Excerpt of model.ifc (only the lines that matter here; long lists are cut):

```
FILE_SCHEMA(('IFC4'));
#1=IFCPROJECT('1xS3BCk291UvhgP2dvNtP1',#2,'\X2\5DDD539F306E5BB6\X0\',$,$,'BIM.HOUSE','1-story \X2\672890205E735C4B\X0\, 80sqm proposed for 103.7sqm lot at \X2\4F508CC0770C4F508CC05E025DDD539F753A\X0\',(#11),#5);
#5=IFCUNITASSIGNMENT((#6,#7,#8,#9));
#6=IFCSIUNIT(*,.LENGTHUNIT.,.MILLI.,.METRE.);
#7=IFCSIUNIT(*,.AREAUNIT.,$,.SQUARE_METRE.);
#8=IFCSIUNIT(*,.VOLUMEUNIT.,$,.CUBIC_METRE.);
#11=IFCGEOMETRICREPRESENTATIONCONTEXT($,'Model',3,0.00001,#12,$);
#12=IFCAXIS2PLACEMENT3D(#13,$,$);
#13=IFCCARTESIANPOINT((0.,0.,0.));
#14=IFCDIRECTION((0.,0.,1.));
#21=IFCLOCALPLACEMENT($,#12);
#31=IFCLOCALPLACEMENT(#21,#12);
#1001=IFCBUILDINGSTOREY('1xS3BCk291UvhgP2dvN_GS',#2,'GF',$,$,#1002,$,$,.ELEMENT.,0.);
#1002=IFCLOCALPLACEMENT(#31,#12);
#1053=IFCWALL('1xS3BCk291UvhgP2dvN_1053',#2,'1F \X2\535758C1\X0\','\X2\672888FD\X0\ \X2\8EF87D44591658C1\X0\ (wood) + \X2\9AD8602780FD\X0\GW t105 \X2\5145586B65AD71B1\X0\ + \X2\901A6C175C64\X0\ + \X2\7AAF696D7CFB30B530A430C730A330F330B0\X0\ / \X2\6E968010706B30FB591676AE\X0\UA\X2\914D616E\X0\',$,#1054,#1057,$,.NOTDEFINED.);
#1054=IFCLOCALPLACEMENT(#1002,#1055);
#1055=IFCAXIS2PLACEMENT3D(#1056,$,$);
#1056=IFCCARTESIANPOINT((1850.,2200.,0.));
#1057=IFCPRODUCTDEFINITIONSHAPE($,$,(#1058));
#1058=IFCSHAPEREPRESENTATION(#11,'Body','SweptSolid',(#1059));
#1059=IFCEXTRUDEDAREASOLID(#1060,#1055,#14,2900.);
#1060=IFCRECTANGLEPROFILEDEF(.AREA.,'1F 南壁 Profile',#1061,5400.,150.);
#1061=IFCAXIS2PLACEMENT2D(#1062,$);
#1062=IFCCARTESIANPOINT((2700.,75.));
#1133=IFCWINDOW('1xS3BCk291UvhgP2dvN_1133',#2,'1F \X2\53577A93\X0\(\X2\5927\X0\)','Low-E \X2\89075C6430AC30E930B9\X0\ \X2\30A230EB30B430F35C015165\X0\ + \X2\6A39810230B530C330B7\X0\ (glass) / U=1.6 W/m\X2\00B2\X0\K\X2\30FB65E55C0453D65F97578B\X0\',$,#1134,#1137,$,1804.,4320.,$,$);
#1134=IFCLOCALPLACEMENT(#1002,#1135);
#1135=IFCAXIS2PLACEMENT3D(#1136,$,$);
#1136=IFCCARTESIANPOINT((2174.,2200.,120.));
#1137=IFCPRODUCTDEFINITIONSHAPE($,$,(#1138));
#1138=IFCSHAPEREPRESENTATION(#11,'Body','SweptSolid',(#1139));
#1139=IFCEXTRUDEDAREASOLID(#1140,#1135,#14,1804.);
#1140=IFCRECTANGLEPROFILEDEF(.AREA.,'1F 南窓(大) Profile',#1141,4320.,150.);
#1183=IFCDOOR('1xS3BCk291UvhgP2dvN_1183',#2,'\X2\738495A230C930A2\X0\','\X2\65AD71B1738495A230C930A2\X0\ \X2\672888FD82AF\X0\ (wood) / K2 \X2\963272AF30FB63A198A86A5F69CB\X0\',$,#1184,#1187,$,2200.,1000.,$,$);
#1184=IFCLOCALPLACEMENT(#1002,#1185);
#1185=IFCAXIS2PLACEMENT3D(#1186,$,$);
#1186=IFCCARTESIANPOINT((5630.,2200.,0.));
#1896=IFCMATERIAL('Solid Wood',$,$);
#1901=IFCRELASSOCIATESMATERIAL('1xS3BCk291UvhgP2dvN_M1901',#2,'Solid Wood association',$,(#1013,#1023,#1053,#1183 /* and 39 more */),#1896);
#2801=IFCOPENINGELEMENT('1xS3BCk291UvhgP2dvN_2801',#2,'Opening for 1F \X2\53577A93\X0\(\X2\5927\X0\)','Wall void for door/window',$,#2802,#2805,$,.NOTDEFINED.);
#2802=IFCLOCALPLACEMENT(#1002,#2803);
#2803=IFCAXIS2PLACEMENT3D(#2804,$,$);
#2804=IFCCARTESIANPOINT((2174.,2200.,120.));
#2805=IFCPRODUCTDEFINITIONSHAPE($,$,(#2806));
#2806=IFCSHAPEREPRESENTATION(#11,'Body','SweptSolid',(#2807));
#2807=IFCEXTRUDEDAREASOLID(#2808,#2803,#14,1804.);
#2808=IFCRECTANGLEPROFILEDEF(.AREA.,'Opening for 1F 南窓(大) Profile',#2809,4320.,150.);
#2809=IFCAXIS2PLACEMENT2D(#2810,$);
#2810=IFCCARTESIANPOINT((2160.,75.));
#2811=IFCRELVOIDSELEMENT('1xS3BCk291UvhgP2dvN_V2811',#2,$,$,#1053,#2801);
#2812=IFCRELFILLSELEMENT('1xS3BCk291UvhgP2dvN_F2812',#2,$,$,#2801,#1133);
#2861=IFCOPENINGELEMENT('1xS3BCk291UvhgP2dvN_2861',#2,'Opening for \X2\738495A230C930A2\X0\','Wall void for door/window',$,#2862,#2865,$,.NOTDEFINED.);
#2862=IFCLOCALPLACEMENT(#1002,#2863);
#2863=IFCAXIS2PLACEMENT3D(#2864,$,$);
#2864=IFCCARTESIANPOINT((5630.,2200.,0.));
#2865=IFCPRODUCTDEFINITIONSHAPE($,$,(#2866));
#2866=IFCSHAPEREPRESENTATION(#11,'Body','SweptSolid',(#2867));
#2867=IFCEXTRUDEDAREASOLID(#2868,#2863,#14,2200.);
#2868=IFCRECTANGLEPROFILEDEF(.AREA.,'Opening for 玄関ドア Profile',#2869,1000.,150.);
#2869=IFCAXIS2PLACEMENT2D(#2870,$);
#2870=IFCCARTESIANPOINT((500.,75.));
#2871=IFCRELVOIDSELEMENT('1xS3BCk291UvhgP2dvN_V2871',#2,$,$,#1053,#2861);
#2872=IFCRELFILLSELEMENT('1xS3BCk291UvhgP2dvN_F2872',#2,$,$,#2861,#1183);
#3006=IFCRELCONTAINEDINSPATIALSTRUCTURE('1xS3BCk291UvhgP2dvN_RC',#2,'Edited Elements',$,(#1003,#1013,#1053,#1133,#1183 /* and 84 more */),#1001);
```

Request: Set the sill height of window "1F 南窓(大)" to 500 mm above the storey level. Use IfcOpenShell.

```python
import numpy as np
import ifcopenshell
import ifcopenshell.api.geometry
import ifcopenshell.geom
import ifcopenshell.util.element
import ifcopenshell.util.placement
import ifcopenshell.util.shape
import ifcopenshell.util.unit

model = ifcopenshell.open("model.ifc")
unit_scale = ifcopenshell.util.unit.calculate_unit_scale(model)

window = model.by_guid("1xS3BCk291UvhgP2dvN_1133")
opening = window.FillsVoids[0].RelatingOpeningElement
storey = ifcopenshell.util.element.get_container(window, ifc_class="IfcBuildingStorey")
level = ifcopenshell.util.placement.get_local_placement(storey.ObjectPlacement)[2, 3]

# The opening's origin need not be at the sill, so measure its lowest point.
shape = ifcopenshell.geom.create_shape(ifcopenshell.geom.settings(), opening)
bottom = ifcopenshell.util.shape.get_shape_bottom_elevation(shape, shape.geometry) / unit_scale
dz = level + 0.5 / unit_scale - bottom

shift = np.array([0.0, 0.0, dz])
# The window is not placed relative to its opening, so move both.
for product in (opening, window):
    matrix = ifcopenshell.util.placement.get_local_placement(product.ObjectPlacement)
    matrix[:3, 3] += shift
    ifcopenshell.api.geometry.edit_object_placement(model, product=product, matrix=matrix, is_si=False)

print(f"moved by {dz * unit_scale:+.3f} m")

model.write("model_edited.ifc")
```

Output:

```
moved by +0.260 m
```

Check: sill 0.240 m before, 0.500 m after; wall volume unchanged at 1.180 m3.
